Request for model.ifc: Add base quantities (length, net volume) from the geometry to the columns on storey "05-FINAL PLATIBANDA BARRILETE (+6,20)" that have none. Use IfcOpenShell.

First a look at what the model holds.

```python
import ifcopenshell
import ifcopenshell.util.element
import ifcopenshell.util.unit

model = ifcopenshell.open("model.ifc")
print(model.schema)
for unit_type in ("LENGTHUNIT", "AREAUNIT", "VOLUMEUNIT"):
    print(unit_type, ifcopenshell.util.unit.calculate_unit_scale(model, unit_type))
storey = next(s for s in model.by_type("IfcBuildingStorey") if s.Name == "05-FINAL PLATIBANDA BARRILETE (+6,20)")
columns = [e for e in ifcopenshell.util.element.get_decomposition(storey) if e.is_a("IfcColumn")]
for e in sorted(columns, key=lambda e: e.id()):
    print(e.id(), e.is_a(), e.Name, list(ifcopenshell.util.element.get_psets(e, qtos_only=True)), sep=" | ")
```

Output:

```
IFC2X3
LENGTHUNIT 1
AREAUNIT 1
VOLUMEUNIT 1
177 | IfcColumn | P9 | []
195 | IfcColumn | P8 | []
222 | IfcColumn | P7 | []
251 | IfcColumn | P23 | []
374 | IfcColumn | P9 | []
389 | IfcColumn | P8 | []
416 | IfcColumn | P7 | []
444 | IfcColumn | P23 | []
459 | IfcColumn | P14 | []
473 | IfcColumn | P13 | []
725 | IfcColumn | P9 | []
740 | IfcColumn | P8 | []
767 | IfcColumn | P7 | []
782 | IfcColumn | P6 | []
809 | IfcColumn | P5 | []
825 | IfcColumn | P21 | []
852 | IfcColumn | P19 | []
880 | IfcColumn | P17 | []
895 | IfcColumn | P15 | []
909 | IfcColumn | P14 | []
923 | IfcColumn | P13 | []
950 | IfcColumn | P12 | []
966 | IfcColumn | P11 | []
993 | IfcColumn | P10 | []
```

```python
import ifcopenshell
import ifcopenshell.api.pset
import ifcopenshell.geom
import ifcopenshell.util.element
import ifcopenshell.util.shape
import ifcopenshell.util.unit

model = ifcopenshell.open("model.ifc")
unit_scale = ifcopenshell.util.unit.calculate_unit_scale(model)
volume_scale = ifcopenshell.util.unit.calculate_unit_scale(model, "VOLUMEUNIT")
settings = ifcopenshell.geom.settings()

storey = next(s for s in model.by_type("IfcBuildingStorey") if s.Name == "05-FINAL PLATIBANDA BARRILETE (+6,20)")
columns = [e for e in ifcopenshell.util.element.get_decomposition(storey) if e.is_a("IfcColumn")]

for e in sorted(columns, key=lambda e: e.id()):
    if ifcopenshell.util.element.get_psets(e, qtos_only=True, should_inherit=False):
        continue
    # Geometry comes back in metres, in the element's own axes.
    shape = ifcopenshell.geom.create_shape(settings, e)
    values = {
        "Length": ifcopenshell.util.shape.get_z(shape.geometry) / unit_scale,
        "NetVolume": ifcopenshell.util.shape.get_volume(shape.geometry) / volume_scale,
    }
    qto = ifcopenshell.api.pset.add_qto(model, product=e, name="BaseQuantities")
    ifcopenshell.api.pset.edit_qto(model, qto=qto, properties=values)
    print(e.id(), {k: round(v, 3) for k, v in values.items()})

model.write("model-out.ifc")
```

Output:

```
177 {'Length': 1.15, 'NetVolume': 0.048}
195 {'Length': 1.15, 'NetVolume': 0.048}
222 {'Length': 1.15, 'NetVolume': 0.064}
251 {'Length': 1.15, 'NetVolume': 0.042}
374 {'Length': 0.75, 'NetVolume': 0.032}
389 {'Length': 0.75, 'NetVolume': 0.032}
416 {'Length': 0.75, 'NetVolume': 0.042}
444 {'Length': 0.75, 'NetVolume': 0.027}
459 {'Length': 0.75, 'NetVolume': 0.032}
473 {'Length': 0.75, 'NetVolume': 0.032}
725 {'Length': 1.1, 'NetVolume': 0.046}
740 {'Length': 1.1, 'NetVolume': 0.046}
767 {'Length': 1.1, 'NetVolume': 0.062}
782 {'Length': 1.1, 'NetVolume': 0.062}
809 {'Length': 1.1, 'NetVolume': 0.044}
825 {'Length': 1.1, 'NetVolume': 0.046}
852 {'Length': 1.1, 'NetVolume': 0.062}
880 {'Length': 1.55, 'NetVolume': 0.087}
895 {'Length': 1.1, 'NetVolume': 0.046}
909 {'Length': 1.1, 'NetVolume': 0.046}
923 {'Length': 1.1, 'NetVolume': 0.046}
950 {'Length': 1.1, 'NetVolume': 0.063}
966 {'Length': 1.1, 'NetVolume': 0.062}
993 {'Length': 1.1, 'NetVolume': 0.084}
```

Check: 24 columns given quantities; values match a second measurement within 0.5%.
